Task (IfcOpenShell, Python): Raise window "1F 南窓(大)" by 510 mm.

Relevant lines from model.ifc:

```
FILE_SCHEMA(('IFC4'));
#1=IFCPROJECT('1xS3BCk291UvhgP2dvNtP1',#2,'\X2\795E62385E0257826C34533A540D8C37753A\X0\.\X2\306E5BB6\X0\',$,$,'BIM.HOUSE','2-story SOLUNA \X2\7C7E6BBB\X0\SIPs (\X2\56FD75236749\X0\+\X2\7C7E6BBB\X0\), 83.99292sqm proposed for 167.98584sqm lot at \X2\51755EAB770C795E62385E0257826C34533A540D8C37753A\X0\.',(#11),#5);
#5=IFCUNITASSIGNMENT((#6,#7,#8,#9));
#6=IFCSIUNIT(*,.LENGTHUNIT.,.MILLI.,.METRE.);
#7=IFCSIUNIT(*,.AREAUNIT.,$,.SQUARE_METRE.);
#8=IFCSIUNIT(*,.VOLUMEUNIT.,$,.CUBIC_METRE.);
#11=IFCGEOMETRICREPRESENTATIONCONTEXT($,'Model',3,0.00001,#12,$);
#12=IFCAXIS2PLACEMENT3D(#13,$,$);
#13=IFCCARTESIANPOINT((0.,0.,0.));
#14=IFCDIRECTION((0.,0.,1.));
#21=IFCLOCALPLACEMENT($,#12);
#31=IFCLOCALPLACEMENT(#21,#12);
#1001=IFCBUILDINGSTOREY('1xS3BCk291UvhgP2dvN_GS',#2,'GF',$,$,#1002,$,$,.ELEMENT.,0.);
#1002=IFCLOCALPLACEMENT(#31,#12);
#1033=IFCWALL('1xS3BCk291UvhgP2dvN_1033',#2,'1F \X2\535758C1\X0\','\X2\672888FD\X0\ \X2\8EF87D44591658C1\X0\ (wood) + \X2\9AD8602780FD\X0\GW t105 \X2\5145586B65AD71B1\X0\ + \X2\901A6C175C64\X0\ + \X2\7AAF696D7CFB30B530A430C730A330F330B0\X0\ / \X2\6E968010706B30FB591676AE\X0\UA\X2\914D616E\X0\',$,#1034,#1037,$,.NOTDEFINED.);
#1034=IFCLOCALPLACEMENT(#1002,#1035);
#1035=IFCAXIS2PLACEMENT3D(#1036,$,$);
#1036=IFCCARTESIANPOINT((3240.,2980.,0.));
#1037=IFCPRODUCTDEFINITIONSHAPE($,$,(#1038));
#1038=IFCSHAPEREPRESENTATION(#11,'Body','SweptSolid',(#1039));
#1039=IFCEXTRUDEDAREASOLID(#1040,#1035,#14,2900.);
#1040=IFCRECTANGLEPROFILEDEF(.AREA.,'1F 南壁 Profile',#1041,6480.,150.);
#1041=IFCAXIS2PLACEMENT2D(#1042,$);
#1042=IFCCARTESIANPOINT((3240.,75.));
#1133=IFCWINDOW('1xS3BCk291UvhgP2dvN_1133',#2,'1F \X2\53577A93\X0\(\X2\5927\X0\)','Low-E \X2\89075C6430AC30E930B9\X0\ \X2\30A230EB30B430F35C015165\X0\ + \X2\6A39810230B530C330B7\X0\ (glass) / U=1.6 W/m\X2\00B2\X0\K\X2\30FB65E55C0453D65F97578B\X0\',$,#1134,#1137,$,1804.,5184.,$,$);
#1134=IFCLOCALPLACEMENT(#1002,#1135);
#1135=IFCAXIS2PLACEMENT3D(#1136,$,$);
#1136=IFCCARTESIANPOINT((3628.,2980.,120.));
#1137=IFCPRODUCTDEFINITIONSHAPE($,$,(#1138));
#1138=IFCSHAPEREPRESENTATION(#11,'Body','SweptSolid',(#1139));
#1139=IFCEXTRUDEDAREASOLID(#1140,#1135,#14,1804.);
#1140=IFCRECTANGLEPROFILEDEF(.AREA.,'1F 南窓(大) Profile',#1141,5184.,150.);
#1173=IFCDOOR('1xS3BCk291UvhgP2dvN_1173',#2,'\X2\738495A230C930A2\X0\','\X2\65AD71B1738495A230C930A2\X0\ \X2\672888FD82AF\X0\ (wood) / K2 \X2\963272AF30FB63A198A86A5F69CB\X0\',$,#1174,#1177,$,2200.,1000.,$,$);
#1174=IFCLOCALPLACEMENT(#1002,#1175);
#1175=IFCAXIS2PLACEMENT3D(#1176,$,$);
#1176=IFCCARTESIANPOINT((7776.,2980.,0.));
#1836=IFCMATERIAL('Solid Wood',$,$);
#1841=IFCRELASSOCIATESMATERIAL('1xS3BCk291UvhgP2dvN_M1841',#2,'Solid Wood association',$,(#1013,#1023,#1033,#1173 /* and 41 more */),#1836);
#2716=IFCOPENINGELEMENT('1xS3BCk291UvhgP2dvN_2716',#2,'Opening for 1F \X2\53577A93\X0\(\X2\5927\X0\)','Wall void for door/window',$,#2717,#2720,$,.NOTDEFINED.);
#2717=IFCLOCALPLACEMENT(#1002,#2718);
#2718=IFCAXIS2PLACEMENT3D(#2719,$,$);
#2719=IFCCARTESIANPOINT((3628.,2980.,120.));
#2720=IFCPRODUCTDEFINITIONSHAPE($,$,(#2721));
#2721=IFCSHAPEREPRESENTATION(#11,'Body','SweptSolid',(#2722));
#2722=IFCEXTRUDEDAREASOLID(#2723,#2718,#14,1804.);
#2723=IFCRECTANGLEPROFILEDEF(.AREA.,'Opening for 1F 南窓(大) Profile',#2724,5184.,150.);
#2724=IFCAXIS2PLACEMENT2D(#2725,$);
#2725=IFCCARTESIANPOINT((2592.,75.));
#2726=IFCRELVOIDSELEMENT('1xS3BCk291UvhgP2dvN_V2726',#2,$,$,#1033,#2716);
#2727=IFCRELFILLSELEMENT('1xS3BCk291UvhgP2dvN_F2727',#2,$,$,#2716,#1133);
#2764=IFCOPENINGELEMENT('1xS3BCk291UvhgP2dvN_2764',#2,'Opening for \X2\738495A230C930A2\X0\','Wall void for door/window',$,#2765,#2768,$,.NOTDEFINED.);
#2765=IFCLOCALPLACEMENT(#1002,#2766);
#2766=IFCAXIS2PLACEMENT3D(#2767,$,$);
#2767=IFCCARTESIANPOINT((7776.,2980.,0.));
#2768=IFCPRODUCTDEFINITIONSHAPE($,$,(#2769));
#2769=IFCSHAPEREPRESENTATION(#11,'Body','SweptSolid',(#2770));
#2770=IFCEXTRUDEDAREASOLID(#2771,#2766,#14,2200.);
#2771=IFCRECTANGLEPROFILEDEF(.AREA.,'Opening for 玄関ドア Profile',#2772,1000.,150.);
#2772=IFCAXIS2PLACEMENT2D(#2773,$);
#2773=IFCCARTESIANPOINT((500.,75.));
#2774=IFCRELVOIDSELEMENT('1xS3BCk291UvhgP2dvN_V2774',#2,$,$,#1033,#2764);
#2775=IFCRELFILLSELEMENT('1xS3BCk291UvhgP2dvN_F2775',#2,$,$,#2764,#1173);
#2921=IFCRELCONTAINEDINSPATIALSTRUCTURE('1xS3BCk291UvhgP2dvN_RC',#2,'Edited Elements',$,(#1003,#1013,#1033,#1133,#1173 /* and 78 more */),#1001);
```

```python
import numpy as np
import ifcopenshell
import ifcopenshell.api.geometry
import ifcopenshell.util.placement
import ifcopenshell.util.unit

model = ifcopenshell.open("model.ifc")
unit_scale = ifcopenshell.util.unit.calculate_unit_scale(model)

window = model.by_id(1133)
opening = window.FillsVoids[0].RelatingOpeningElement
dz = 0.51 / unit_scale

shift = np.array([0.0, 0.0, dz])
# The window is not placed relative to its opening, so move both.
for product in (opening, window):
    matrix = ifcopenshell.util.placement.get_local_placement(product.ObjectPlacement)
    matrix[:3, 3] += shift
    ifcopenshell.api.geometry.edit_object_placement(model, product=product, matrix=matrix, is_si=False)

print(f"moved by {dz * unit_scale:+.3f} m")

model.write("model_v2.ifc")
```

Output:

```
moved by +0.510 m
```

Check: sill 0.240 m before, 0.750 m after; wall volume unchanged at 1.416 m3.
